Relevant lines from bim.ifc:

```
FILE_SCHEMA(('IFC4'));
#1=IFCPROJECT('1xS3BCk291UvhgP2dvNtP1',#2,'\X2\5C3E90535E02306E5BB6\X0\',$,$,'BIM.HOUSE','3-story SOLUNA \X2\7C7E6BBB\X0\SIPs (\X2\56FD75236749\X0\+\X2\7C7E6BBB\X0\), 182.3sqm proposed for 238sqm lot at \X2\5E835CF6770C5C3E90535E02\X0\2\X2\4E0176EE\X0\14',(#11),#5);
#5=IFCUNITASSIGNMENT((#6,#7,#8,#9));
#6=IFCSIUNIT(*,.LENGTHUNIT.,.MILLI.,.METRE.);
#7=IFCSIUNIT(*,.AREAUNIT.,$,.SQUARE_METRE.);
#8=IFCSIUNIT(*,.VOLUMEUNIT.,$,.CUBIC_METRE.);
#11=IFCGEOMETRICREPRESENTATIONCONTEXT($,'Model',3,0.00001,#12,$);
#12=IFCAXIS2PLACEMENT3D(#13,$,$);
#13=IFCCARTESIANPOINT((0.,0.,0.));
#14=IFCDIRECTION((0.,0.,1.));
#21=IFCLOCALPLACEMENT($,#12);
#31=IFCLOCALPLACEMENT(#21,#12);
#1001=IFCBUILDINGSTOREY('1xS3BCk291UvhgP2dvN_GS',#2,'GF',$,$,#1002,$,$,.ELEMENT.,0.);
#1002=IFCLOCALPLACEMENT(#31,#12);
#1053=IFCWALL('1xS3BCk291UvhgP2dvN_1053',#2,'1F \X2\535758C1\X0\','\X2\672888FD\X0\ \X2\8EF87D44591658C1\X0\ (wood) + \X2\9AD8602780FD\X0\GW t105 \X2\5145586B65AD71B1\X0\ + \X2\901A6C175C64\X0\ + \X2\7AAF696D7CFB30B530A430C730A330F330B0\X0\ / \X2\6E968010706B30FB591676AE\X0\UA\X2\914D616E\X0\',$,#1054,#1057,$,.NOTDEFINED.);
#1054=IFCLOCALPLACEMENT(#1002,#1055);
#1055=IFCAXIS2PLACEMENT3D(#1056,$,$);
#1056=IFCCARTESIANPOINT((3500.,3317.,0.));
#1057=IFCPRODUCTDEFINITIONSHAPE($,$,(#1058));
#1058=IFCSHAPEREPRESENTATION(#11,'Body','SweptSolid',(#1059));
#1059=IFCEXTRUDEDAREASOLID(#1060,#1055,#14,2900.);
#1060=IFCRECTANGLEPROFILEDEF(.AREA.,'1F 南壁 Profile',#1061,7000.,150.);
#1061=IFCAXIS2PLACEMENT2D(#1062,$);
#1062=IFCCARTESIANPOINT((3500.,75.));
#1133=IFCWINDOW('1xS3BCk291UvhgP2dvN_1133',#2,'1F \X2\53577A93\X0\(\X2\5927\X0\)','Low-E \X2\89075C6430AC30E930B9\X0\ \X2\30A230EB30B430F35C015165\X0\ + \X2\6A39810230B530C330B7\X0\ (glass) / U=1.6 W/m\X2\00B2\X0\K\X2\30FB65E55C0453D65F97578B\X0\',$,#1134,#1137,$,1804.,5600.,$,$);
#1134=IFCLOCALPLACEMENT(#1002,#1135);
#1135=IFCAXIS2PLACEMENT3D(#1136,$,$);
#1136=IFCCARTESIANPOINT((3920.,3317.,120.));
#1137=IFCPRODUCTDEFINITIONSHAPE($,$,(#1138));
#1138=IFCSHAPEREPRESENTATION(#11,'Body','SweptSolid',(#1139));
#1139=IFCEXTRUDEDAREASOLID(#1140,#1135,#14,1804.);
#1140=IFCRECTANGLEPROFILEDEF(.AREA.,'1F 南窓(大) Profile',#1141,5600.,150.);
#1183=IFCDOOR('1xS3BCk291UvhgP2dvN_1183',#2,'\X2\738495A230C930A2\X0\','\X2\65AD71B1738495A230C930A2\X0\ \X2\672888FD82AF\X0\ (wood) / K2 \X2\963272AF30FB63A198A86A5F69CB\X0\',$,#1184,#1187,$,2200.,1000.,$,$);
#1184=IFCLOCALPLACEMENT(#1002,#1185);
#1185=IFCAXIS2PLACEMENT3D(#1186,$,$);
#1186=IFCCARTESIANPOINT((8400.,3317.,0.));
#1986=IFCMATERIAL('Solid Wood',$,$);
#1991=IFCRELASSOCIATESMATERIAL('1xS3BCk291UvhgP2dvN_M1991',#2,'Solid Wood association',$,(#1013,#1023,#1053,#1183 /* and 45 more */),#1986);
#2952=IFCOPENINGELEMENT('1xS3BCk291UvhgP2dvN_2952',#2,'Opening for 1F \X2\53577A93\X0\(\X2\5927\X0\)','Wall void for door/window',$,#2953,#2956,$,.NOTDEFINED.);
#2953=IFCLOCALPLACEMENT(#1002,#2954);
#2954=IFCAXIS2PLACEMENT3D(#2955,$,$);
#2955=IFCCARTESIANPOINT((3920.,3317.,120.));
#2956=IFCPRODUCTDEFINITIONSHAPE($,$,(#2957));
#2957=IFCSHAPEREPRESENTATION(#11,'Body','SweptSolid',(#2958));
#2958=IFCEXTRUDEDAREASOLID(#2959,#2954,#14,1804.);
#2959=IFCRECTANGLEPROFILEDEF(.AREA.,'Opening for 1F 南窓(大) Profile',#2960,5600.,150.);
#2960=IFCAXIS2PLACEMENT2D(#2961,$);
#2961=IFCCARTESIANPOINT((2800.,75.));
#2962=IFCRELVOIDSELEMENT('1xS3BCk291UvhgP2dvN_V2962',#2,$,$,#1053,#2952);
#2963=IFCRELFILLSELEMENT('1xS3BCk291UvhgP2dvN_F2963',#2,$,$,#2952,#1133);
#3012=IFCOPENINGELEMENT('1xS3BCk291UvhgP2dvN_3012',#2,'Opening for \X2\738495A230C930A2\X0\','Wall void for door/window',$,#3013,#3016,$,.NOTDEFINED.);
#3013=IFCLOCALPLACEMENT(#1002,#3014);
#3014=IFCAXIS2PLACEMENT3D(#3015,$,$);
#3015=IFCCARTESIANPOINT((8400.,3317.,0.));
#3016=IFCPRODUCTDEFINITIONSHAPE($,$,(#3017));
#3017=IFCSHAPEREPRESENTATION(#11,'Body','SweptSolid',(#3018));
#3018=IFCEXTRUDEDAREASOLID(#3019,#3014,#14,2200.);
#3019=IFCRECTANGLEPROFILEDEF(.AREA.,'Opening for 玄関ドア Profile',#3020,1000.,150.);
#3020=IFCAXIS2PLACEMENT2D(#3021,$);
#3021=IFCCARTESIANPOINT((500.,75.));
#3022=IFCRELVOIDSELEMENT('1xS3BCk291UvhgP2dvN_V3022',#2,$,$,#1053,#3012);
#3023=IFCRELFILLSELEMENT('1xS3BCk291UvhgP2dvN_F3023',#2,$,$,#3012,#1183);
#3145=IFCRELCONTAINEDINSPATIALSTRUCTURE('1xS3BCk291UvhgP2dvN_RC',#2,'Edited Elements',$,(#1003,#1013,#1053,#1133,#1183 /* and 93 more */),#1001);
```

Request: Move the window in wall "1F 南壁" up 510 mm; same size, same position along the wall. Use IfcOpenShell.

```python
import numpy as np
import ifcopenshell
import ifcopenshell.api.geometry
import ifcopenshell.util.placement
import ifcopenshell.util.unit

model = ifcopenshell.open("bim.ifc")
unit_scale = ifcopenshell.util.unit.calculate_unit_scale(model)

window = model.by_guid("1xS3BCk291UvhgP2dvN_1133")
opening = window.FillsVoids[0].RelatingOpeningElement
dz = 0.51 / unit_scale

shift = np.array([0.0, 0.0, dz])
# The window is not placed relative to its opening, so move both.
for product in (opening, window):
    matrix = ifcopenshell.util.placement.get_local_placement(product.ObjectPlacement)
    matrix[:3, 3] += shift
    ifcopenshell.api.geometry.edit_object_placement(model, product=product, matrix=matrix, is_si=False)

print(f"moved by {dz * unit_scale:+.3f} m")

model.write("bim-out.ifc")
```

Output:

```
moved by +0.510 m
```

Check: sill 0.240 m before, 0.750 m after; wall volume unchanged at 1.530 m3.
